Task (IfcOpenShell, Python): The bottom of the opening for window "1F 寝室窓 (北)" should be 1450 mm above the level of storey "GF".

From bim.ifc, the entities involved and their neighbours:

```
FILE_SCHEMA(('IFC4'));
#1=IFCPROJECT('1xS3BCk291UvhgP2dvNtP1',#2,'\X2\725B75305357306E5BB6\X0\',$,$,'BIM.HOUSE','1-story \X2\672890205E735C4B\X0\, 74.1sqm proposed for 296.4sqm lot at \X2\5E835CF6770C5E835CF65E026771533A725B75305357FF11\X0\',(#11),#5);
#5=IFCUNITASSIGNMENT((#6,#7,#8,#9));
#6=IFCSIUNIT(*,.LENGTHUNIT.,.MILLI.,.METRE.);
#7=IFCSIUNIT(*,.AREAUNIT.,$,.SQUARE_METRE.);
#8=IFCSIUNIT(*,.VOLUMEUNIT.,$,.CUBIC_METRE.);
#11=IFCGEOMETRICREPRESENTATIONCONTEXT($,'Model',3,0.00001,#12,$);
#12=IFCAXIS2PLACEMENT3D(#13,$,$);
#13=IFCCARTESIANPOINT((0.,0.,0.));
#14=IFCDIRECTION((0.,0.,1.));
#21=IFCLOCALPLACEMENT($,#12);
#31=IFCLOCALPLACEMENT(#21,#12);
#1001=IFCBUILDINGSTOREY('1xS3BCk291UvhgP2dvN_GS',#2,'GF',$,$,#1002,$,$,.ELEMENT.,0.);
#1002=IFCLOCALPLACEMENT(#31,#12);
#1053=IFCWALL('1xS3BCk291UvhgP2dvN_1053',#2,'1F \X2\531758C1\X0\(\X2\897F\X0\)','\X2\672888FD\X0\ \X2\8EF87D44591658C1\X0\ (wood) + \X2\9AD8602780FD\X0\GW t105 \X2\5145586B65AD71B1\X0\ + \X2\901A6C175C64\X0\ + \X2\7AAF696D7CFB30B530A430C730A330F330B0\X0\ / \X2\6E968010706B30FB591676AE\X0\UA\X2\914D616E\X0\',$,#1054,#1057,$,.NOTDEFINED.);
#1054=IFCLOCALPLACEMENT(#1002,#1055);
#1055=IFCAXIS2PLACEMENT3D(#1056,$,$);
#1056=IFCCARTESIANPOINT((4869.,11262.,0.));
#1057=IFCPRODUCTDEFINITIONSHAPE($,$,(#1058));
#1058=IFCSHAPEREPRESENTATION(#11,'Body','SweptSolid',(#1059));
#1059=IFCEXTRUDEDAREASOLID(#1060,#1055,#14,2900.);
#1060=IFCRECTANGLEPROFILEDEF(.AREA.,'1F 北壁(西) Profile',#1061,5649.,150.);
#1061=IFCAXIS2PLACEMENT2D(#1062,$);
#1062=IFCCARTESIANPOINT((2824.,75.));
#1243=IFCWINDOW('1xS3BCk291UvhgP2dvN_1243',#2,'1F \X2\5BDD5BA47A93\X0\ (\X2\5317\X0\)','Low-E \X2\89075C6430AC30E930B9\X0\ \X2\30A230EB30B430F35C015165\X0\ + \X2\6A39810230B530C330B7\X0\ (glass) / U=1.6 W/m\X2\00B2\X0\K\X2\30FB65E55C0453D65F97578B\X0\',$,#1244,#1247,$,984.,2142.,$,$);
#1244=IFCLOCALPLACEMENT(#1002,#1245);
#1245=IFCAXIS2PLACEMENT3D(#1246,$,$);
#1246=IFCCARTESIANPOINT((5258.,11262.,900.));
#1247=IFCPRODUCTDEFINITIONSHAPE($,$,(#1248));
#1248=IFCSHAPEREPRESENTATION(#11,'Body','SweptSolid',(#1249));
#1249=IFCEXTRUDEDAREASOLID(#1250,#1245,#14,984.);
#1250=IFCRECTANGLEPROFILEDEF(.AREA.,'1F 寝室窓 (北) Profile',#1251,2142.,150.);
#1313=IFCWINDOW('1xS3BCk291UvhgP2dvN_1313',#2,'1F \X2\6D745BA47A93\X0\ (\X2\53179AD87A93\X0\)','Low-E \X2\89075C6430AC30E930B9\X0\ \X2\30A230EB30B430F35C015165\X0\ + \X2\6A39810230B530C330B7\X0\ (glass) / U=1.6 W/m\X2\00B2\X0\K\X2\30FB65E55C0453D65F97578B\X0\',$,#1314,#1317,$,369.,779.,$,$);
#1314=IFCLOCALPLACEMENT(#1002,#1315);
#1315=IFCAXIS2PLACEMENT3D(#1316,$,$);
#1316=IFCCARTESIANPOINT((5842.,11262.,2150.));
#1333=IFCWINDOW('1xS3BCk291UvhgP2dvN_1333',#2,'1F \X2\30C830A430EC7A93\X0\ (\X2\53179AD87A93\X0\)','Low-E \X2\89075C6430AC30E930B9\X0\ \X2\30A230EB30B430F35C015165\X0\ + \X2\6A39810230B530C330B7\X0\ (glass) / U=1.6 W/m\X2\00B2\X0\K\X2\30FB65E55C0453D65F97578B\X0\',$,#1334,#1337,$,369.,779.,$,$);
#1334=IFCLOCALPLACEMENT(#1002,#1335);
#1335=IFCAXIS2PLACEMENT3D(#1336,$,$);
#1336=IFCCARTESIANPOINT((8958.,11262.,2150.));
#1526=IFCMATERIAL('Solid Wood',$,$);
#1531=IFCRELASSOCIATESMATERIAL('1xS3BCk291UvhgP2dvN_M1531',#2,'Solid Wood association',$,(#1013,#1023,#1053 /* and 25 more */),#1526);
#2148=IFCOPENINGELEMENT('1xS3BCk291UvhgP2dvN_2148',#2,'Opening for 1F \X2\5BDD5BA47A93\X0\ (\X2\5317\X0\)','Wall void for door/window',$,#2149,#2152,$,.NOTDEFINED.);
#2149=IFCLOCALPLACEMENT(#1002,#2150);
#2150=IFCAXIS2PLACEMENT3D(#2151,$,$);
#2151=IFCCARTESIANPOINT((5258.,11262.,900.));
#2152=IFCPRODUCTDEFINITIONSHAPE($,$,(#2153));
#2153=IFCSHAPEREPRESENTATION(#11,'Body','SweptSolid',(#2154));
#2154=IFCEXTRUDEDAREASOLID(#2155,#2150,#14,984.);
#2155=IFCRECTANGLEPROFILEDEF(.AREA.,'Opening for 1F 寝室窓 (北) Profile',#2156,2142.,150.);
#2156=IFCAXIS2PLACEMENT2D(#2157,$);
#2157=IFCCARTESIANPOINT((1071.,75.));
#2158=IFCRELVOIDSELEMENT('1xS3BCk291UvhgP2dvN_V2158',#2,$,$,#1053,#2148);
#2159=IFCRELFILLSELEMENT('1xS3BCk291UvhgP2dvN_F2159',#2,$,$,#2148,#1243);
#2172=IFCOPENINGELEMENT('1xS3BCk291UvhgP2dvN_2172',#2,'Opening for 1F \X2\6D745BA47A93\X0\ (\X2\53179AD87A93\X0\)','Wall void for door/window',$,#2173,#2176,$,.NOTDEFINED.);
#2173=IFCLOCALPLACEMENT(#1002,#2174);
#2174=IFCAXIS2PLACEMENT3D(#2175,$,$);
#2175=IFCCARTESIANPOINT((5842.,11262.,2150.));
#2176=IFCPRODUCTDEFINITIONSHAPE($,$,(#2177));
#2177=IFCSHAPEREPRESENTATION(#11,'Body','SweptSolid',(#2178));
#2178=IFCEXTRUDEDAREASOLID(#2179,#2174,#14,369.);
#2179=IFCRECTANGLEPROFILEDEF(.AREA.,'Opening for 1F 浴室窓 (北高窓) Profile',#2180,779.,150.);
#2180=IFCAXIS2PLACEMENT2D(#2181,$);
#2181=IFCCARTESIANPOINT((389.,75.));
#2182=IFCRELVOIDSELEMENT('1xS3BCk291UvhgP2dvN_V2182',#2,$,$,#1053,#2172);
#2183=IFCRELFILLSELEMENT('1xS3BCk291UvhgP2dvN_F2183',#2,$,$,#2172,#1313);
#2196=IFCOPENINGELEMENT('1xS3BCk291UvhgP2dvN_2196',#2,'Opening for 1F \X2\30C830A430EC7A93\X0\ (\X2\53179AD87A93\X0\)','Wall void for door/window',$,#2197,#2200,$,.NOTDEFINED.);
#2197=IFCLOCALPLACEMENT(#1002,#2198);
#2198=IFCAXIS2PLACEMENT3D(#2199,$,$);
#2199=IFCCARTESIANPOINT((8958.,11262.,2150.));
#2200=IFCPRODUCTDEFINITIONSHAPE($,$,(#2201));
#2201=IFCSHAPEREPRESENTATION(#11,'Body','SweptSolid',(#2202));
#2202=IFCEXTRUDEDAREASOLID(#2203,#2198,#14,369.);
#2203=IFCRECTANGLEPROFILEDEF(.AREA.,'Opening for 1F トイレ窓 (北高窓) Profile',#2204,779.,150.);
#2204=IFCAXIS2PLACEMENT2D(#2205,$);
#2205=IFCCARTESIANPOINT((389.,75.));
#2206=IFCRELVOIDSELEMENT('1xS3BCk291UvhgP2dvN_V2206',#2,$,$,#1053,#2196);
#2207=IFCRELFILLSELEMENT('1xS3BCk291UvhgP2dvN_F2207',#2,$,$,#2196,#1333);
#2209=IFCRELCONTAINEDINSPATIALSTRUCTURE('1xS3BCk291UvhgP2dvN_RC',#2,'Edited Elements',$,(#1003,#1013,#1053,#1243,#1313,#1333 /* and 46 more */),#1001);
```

```python
import numpy as np
import ifcopenshell
import ifcopenshell.api.geometry
import ifcopenshell.geom
import ifcopenshell.util.element
import ifcopenshell.util.placement
import ifcopenshell.util.shape
import ifcopenshell.util.unit

model = ifcopenshell.open("bim.ifc")
unit_scale = ifcopenshell.util.unit.calculate_unit_scale(model)

window = model.by_id(1243)
opening = window.FillsVoids[0].RelatingOpeningElement
storey = ifcopenshell.util.element.get_container(window, ifc_class="IfcBuildingStorey")
level = ifcopenshell.util.placement.get_local_placement(storey.ObjectPlacement)[2, 3]

# The opening's origin need not be at the sill, so measure its lowest point.
shape = ifcopenshell.geom.create_shape(ifcopenshell.geom.settings(), opening)
bottom = ifcopenshell.util.shape.get_shape_bottom_elevation(shape, shape.geometry) / unit_scale
dz = level + 1.45 / unit_scale - bottom

shift = np.array([0.0, 0.0, dz])
# The window is not placed relative to its opening, so move both.
for product in (opening, window):
    matrix = ifcopenshell.util.placement.get_local_placement(product.ObjectPlacement)
    matrix[:3, 3] += shift
    ifcopenshell.api.geometry.edit_object_placement(model, product=product, matrix=matrix, is_si=False)

print(f"moved by {dz * unit_scale:+.3f} m")

model.write("bim_rev.ifc")
```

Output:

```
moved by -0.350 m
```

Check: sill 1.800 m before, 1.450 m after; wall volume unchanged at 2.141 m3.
